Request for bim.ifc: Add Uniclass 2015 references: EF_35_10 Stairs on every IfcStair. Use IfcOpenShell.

First a look at what the model holds.

```python
import ifcopenshell

model = ifcopenshell.open("bim.ifc")
print(model.schema)
print("classifications:", [c.Name for c in model.by_type("IfcClassification")])
for ifc_class in ("IfcDoor", "IfcRoof", "IfcStair", "IfcWall", "IfcWindow"):
    print(ifc_class, len(model.by_type(ifc_class)))
```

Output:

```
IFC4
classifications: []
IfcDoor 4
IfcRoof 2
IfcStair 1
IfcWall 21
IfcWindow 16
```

```python
import ifcopenshell
import ifcopenshell.api.classification

model = ifcopenshell.open("bim.ifc")

system = ifcopenshell.api.classification.add_classification(model, classification="Uniclass 2015")

codes = {
    "IfcStair": ("EF_35_10", "Stairs"),
}
for ifc_class, (code, name) in codes.items():
    products = model.by_type(ifc_class)
    ifcopenshell.api.classification.add_reference(
        model, products=products, classification=system, identification=code, name=name
    )
    print(code, len(products))

model.write("bim_updated.ifc")
```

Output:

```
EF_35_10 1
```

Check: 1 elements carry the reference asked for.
